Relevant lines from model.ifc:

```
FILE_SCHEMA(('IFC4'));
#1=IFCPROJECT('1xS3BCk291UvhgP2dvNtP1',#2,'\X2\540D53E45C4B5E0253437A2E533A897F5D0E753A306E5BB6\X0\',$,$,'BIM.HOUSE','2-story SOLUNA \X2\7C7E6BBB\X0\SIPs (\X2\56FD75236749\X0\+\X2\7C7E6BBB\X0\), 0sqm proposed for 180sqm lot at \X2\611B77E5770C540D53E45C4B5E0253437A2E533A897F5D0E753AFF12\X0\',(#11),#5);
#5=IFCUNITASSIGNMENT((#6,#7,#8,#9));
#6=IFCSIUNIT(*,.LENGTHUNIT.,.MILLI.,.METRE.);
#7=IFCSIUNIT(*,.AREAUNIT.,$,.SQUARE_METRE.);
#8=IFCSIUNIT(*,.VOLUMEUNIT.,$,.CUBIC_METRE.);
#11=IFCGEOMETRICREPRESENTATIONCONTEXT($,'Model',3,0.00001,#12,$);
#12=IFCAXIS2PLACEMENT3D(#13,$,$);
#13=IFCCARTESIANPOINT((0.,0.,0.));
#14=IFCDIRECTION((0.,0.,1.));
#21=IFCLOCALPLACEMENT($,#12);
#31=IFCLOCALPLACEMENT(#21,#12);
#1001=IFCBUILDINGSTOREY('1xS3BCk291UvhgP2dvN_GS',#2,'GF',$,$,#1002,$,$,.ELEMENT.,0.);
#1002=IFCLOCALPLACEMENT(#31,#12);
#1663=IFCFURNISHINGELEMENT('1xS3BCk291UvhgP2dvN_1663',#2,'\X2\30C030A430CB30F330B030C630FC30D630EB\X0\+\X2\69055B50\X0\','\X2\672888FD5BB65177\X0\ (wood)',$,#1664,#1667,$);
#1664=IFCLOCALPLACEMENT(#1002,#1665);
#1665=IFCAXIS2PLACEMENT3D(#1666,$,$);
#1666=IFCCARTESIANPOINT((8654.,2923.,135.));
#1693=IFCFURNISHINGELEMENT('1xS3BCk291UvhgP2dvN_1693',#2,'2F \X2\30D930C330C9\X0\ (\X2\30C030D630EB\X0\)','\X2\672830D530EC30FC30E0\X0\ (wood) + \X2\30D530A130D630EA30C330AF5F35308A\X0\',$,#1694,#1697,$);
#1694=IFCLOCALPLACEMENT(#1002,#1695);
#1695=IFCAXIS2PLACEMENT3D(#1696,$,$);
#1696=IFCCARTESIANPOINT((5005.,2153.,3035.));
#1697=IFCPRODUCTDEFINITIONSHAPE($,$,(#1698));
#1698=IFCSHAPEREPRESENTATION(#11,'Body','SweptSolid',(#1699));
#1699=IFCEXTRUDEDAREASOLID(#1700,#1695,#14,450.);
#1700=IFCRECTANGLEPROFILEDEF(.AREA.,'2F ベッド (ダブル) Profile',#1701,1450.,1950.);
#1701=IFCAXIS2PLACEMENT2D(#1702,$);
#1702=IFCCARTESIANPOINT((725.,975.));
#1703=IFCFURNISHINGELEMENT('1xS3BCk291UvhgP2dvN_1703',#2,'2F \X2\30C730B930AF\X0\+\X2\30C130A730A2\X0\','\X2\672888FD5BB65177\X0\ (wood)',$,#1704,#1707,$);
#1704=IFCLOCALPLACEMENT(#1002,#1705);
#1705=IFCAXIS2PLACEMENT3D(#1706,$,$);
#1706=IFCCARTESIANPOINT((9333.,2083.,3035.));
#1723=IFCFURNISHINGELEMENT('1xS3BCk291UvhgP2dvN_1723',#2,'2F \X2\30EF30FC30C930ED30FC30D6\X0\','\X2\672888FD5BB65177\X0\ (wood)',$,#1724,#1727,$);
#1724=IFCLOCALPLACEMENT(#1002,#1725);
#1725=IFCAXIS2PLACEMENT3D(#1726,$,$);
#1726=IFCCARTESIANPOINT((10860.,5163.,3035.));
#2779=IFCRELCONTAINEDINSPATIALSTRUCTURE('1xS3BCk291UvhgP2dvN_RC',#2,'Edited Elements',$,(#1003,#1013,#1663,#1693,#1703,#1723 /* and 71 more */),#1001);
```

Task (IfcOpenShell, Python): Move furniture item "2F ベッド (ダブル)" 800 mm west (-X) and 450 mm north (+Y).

```python
import ifcopenshell
import ifcopenshell.api.geometry
import ifcopenshell.util.placement
import ifcopenshell.util.unit

model = ifcopenshell.open("model.ifc")
unit_scale = ifcopenshell.util.unit.calculate_unit_scale(model)

item = model.by_guid("1xS3BCk291UvhgP2dvN_1693")
matrix = ifcopenshell.util.placement.get_local_placement(item.ObjectPlacement)
matrix[0, 3] -= 0.8 / unit_scale
matrix[1, 3] += 0.45 / unit_scale
ifcopenshell.api.geometry.edit_object_placement(model, product=item, matrix=matrix, is_si=False)

print(ifcopenshell.util.placement.get_local_placement(item.ObjectPlacement).round(3) + 0.0)

model.write("model_updated.ifc")
```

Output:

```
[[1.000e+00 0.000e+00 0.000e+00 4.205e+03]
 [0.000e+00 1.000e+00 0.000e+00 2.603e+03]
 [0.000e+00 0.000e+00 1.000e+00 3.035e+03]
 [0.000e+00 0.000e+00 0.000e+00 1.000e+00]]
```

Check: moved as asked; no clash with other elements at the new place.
